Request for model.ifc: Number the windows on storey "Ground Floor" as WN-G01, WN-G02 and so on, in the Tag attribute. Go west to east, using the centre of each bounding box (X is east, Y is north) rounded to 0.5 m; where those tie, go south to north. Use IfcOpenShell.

First a look at what the model holds.

```python
import ifcopenshell
import ifcopenshell.util.element
import ifcopenshell.util.placement

model = ifcopenshell.open("model.ifc")
print(model.schema)
storey = next(s for s in model.by_type("IfcBuildingStorey") if s.Name == "Ground Floor")
windows = [e for e in ifcopenshell.util.element.get_decomposition(storey) if e.is_a("IfcWindow")]
for e in sorted(windows, key=lambda e: e.id()):
    origin = ifcopenshell.util.placement.get_local_placement(e.ObjectPlacement)[:3, 3]
    print(e.id(), e.Tag, e.Name, origin.round(2) + 0.0, sep=" | ")
```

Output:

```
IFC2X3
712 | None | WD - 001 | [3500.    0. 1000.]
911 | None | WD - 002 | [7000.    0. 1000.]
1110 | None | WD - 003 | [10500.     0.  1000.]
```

```python
import ifcopenshell
import ifcopenshell.geom
import ifcopenshell.util.element
import ifcopenshell.util.shape

model = ifcopenshell.open("model.ifc")
settings = ifcopenshell.geom.settings()
settings.set("use-world-coords", True)


def centre(element):
    shape = ifcopenshell.geom.create_shape(settings, element)
    return ifcopenshell.util.shape.get_bbox_centroid(shape.geometry)


storey = next(s for s in model.by_type("IfcBuildingStorey") if s.Name == "Ground Floor")
windows = [e for e in ifcopenshell.util.element.get_decomposition(storey) if e.is_a("IfcWindow")]

# Insertion points can sit at a corner or the storey origin, so sort by the geometry (in metres).
centres = {e: centre(e) for e in windows}
windows.sort(key=lambda e: (round(centres[e][0] / 0.5), centres[e][1]))

for i, e in enumerate(windows, start=1):
    number = f"WN-G{i:02d}"
    e.Tag = number
    print(e.id(), number)

model.write("model_updated.ifc")
```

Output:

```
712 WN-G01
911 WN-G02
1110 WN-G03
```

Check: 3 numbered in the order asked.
